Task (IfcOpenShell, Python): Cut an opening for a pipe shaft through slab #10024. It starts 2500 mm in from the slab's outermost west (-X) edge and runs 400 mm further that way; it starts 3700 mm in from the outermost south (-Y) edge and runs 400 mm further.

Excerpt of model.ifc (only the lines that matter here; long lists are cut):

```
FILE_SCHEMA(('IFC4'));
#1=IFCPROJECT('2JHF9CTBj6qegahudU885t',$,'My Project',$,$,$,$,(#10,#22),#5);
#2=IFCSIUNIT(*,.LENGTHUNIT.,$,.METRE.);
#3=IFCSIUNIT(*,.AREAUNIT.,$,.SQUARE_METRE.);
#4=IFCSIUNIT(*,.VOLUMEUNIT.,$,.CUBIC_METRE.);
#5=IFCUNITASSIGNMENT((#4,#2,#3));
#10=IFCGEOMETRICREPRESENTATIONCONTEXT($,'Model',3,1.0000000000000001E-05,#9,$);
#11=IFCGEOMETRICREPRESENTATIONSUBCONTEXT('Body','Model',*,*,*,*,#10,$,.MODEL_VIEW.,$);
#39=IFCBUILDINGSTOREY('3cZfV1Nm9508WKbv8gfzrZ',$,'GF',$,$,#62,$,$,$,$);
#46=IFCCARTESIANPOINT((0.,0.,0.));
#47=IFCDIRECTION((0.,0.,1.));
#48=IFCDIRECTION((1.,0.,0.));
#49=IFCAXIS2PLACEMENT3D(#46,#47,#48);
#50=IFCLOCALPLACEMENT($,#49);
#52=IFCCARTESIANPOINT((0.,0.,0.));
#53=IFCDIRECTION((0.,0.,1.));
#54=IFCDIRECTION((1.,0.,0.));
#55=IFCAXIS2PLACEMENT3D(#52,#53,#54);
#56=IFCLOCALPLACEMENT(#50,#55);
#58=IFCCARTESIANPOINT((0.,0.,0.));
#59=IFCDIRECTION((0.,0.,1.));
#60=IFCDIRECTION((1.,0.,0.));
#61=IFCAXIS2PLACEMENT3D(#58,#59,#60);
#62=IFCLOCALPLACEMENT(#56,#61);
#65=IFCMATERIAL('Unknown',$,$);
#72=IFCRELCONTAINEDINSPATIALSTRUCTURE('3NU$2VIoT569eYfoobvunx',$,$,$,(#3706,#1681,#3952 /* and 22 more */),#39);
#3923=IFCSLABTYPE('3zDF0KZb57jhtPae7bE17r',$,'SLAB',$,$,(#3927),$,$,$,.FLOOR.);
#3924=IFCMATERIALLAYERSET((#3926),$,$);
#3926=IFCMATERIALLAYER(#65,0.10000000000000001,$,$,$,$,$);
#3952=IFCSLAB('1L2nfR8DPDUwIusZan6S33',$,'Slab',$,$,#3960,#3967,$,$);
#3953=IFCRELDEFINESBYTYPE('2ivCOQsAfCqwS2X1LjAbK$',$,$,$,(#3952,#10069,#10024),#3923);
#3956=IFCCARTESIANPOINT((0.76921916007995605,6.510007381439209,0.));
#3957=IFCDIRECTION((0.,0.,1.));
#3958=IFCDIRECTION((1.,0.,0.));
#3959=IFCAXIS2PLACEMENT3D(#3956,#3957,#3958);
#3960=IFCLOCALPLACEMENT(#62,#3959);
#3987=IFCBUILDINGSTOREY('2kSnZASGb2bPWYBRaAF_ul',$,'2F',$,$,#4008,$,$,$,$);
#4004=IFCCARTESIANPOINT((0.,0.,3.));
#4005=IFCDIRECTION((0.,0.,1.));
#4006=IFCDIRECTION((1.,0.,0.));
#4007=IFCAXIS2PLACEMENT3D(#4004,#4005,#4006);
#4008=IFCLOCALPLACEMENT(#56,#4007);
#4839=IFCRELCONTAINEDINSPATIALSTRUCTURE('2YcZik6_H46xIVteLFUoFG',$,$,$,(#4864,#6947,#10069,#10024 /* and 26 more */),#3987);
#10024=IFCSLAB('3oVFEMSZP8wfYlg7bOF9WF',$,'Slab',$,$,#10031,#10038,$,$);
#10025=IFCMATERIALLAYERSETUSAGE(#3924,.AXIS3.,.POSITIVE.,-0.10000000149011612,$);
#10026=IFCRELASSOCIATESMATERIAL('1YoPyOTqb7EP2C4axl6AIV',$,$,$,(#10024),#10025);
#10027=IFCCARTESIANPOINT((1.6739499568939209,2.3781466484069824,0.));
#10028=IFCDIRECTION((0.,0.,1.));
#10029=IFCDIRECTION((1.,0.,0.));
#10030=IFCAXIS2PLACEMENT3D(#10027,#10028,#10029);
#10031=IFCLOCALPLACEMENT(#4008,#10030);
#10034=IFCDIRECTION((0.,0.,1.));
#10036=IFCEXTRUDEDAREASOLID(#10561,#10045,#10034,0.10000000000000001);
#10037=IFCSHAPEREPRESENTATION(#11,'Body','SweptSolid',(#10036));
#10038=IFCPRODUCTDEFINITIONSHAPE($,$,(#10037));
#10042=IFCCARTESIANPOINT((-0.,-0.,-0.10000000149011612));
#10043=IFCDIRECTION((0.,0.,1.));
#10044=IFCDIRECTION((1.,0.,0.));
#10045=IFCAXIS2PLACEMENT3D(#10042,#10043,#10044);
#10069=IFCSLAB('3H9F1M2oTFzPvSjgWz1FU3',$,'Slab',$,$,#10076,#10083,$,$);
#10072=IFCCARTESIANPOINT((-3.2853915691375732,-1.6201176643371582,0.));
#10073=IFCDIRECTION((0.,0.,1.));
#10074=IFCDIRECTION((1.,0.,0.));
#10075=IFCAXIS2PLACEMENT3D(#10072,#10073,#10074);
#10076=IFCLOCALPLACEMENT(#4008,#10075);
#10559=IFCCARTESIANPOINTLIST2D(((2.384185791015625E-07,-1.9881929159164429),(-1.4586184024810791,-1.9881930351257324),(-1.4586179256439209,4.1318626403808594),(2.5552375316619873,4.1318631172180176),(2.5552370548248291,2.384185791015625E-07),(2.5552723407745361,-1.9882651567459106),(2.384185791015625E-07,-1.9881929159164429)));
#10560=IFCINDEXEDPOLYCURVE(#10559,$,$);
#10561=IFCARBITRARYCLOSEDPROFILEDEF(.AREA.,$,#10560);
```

```python
import numpy as np
import ifcopenshell
import ifcopenshell.api.feature
import ifcopenshell.api.geometry
import ifcopenshell.api.root
import ifcopenshell.geom
import ifcopenshell.util.placement
import ifcopenshell.util.representation
import ifcopenshell.util.shape
import ifcopenshell.util.unit

model = ifcopenshell.open("model.ifc")
unit_scale = ifcopenshell.util.unit.calculate_unit_scale(model)
settings = ifcopenshell.geom.settings()


def volume(element):
    """Net volume in cubic metres, openings subtracted."""
    shape = ifcopenshell.geom.create_shape(settings, element)
    return ifcopenshell.util.shape.get_volume(shape.geometry)


slab = model.by_guid("3oVFEMSZP8wfYlg7bOF9WF")
before = volume(slab)

# Extent in the slab's own axes, in metres. The edges named are its -X and -Y sides.
slab_shape = ifcopenshell.geom.create_shape(settings, slab)
vertices = ifcopenshell.util.shape.get_vertices(slab_shape.geometry)
x_min, y_min, bottom = vertices.min(axis=0)
top = vertices[:, 2].max()

opening = ifcopenshell.api.root.create_entity(model, ifc_class="IfcOpeningElement", name="Pipe shaft opening", predefined_type="OPENING")
context = ifcopenshell.util.representation.get_context(model, "Model", "Body", "MODEL_VIEW")
width, depth = 0.4, 0.4
outline = [(0.0, 0.0), (width, 0.0), (width, depth), (0.0, depth), (0.0, 0.0)]
# Overshoot both faces by 50 mm so the cut is clean.
shape = ifcopenshell.api.geometry.add_slab_representation(
    model, context=context, depth=top - bottom + 0.1, polyline=outline
)
ifcopenshell.api.geometry.assign_representation(model, product=opening, representation=shape)

matrix = ifcopenshell.util.placement.get_local_placement(slab.ObjectPlacement)
matrix[:, 3] = matrix @ np.append(np.array([x_min + 2.5, y_min + 3.7, bottom - 0.05]) / unit_scale, 1.0)
ifcopenshell.api.geometry.edit_object_placement(model, product=opening, matrix=matrix, is_si=False)
ifcopenshell.api.feature.add_feature(model, feature=opening, element=slab)

after = volume(slab)

print(f"slab volume {before:.3f} -> {after:.3f} m3")

model.write("model_rev.ifc")
```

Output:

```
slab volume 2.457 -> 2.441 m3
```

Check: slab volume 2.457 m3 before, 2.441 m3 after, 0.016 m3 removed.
